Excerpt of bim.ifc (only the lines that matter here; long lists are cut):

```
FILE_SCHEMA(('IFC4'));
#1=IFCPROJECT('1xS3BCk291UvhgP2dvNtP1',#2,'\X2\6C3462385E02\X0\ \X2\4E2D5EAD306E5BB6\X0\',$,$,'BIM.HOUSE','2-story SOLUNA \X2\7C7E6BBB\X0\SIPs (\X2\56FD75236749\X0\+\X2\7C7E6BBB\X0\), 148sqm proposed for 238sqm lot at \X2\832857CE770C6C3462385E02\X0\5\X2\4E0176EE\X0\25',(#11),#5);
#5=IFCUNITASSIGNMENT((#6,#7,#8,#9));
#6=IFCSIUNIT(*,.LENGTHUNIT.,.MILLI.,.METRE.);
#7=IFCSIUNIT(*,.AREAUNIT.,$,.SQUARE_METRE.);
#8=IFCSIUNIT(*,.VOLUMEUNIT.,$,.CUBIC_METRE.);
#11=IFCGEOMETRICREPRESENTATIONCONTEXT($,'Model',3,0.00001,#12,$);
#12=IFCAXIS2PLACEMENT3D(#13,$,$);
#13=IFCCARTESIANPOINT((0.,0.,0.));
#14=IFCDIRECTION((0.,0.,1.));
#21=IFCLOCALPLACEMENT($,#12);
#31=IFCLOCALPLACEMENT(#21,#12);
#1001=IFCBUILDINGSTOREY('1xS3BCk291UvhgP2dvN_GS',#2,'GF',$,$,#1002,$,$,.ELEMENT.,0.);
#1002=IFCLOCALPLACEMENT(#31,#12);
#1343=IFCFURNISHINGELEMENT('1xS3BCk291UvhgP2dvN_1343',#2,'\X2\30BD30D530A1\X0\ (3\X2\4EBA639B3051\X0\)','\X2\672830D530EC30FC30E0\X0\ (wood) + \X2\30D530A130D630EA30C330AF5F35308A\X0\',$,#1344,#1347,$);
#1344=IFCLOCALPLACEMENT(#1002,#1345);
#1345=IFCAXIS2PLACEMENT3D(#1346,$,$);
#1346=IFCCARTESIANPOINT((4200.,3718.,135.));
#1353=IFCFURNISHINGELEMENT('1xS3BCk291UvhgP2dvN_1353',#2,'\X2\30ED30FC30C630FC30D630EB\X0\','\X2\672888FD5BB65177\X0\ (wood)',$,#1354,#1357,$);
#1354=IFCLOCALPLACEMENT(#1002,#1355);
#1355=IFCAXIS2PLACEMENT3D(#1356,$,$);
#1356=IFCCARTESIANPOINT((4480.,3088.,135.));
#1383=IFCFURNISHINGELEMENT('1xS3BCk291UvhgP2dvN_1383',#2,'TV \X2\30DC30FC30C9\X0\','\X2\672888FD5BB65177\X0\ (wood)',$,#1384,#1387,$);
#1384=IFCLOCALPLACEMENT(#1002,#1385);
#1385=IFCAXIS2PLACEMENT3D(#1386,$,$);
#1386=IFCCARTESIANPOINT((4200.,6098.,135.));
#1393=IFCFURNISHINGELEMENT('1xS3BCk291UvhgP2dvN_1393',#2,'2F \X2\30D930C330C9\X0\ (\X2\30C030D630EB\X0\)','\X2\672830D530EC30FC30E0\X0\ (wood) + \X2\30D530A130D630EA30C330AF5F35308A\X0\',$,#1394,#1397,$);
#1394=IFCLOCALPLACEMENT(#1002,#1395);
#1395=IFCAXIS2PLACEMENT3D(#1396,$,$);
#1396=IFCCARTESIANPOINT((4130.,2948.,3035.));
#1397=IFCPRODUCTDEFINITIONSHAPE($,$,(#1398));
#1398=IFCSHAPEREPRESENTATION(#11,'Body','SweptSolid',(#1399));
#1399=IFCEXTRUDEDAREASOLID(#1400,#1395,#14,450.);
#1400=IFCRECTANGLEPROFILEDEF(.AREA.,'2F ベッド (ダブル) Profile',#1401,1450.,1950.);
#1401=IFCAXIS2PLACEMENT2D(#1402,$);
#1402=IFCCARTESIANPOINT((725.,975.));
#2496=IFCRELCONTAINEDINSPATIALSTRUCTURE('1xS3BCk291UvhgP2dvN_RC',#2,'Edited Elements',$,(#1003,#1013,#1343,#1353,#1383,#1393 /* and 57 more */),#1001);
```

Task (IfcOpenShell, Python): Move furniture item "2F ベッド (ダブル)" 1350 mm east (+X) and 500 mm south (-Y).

```python
import ifcopenshell
import ifcopenshell.api.geometry
import ifcopenshell.util.placement

model = ifcopenshell.open("bim.ifc")

item = model.by_guid("1xS3BCk291UvhgP2dvN_1393")
matrix = ifcopenshell.util.placement.get_local_placement(item.ObjectPlacement)
matrix[0, 3] += 1350.0
matrix[1, 3] -= 500.0
ifcopenshell.api.geometry.edit_object_placement(model, product=item, matrix=matrix, is_si=False)

print(ifcopenshell.util.placement.get_local_placement(item.ObjectPlacement).round(3) + 0.0)

model.write("bim_v2.ifc")
```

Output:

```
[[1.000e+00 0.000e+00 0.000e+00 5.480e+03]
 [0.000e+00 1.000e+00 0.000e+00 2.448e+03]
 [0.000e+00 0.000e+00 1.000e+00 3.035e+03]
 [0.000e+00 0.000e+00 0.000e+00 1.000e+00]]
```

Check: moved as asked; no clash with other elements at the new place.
